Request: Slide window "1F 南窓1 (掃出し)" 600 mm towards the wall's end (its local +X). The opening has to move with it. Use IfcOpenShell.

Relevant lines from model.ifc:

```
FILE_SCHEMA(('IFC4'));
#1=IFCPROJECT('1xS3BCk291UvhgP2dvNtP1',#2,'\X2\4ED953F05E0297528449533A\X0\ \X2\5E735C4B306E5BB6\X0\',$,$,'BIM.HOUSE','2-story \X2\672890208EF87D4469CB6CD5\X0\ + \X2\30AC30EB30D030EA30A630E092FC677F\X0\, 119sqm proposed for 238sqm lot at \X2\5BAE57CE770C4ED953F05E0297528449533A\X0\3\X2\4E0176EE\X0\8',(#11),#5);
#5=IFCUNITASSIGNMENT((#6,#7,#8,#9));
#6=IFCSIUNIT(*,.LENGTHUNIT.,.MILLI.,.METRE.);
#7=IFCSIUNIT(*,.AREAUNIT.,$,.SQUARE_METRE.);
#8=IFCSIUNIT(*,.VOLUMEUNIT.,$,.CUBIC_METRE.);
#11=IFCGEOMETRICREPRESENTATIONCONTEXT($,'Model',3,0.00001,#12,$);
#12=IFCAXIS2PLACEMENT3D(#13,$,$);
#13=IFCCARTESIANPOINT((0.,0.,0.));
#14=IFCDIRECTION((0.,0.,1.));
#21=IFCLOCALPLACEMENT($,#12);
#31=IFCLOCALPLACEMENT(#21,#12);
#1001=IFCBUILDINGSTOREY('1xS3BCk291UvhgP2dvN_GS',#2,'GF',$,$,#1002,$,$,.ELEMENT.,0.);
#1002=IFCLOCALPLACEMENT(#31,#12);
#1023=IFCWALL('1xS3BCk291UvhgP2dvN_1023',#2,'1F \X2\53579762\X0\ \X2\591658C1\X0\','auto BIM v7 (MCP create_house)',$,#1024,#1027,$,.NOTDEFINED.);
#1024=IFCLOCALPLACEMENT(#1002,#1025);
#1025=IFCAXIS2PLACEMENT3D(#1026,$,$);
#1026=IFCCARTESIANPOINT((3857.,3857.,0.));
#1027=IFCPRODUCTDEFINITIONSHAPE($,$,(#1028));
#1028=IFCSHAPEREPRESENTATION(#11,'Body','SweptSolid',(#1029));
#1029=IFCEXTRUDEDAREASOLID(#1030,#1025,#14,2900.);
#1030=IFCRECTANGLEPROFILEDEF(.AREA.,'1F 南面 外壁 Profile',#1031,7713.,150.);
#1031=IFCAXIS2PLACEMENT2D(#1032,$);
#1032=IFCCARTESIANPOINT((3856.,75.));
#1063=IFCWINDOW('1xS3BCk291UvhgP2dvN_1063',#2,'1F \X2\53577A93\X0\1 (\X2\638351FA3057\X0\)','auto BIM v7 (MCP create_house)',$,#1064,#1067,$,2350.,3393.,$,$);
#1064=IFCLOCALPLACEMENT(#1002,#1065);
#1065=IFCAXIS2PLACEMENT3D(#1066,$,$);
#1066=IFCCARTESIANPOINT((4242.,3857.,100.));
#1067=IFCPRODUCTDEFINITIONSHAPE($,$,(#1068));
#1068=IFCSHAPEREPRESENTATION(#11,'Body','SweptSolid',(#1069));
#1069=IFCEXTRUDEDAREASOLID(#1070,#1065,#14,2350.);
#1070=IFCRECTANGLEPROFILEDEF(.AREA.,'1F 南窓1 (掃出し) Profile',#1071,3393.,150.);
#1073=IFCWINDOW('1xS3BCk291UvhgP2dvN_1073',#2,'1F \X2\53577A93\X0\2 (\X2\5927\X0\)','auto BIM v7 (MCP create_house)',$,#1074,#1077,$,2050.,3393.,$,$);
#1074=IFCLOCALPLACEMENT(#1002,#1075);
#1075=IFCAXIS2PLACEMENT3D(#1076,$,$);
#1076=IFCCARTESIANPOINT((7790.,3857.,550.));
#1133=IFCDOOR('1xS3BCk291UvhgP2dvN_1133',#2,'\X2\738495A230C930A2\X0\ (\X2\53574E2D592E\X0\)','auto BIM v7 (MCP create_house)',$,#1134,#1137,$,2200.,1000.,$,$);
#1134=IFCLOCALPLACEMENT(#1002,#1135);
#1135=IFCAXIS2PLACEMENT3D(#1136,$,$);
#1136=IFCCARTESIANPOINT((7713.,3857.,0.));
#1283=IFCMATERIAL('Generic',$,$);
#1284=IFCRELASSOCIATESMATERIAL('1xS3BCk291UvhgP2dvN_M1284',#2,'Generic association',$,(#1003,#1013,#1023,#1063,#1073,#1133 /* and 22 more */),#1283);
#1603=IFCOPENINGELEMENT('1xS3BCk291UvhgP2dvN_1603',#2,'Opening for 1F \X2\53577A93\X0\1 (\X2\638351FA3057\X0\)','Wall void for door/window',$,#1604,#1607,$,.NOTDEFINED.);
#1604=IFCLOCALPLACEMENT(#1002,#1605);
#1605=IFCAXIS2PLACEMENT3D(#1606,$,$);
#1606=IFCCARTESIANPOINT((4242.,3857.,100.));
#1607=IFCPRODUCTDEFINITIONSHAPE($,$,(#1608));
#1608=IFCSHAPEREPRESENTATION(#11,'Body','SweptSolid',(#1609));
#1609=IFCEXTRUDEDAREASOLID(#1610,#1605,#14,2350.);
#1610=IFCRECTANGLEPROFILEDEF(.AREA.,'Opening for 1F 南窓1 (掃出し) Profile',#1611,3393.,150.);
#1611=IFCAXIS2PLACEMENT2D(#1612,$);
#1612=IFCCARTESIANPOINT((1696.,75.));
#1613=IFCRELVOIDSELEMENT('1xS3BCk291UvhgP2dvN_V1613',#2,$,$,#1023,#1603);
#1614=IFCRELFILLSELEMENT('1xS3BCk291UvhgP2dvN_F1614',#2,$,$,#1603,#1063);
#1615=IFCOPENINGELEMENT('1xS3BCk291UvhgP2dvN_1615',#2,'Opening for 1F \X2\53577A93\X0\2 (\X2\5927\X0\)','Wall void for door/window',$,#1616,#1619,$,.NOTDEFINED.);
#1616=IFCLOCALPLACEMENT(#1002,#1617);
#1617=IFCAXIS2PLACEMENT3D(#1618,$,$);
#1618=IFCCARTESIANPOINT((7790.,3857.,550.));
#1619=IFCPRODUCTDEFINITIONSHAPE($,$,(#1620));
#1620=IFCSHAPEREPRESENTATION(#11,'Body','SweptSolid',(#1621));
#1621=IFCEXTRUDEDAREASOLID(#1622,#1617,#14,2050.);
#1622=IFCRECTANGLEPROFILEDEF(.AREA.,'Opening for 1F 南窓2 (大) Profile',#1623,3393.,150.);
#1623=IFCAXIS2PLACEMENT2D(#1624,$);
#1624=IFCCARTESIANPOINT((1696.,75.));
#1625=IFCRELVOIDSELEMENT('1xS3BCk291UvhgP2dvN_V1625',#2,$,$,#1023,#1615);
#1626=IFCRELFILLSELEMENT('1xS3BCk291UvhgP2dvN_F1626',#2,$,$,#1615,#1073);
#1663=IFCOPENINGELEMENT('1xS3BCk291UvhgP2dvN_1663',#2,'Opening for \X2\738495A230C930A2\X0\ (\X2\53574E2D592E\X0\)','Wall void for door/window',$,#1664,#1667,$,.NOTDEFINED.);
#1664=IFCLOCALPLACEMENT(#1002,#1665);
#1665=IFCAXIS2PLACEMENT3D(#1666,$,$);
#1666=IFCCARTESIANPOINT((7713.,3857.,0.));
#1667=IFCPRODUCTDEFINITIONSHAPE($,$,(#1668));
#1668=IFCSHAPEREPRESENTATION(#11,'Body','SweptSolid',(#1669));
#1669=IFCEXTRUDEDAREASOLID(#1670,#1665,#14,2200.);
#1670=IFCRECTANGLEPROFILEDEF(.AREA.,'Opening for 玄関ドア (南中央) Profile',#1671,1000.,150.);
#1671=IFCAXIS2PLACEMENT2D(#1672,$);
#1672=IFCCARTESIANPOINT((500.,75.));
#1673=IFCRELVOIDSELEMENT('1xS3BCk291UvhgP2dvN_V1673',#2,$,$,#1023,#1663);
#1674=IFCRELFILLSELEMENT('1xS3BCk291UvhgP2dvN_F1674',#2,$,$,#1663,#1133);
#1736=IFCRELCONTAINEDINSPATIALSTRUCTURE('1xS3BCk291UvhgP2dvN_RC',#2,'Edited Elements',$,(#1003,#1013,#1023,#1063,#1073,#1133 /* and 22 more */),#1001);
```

```python
import ifcopenshell
import ifcopenshell.api.geometry
import ifcopenshell.util.placement
import ifcopenshell.util.unit

model = ifcopenshell.open("model.ifc")
unit_scale = ifcopenshell.util.unit.calculate_unit_scale(model)

window = model.by_id(1063)
opening = window.FillsVoids[0].RelatingOpeningElement
wall = opening.VoidsElements[0].RelatingBuildingElement

wall_matrix = ifcopenshell.util.placement.get_local_placement(wall.ObjectPlacement)
shift = wall_matrix[:3, 0] * 0.6 / unit_scale
before = ifcopenshell.util.placement.get_local_placement(window.ObjectPlacement)[:3, 3].copy()

# The window is not placed relative to its opening, so move both.
for product in (opening, window):
    matrix = ifcopenshell.util.placement.get_local_placement(product.ObjectPlacement)
    matrix[:3, 3] += shift
    ifcopenshell.api.geometry.edit_object_placement(model, product=product, matrix=matrix, is_si=False)

after = ifcopenshell.util.placement.get_local_placement(window.ObjectPlacement)[:3, 3]
print("window moved by", (after - before).round(3) + 0.0)

model.write("model_v2.ifc")
```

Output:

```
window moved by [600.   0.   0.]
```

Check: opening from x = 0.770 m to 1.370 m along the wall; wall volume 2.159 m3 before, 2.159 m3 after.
